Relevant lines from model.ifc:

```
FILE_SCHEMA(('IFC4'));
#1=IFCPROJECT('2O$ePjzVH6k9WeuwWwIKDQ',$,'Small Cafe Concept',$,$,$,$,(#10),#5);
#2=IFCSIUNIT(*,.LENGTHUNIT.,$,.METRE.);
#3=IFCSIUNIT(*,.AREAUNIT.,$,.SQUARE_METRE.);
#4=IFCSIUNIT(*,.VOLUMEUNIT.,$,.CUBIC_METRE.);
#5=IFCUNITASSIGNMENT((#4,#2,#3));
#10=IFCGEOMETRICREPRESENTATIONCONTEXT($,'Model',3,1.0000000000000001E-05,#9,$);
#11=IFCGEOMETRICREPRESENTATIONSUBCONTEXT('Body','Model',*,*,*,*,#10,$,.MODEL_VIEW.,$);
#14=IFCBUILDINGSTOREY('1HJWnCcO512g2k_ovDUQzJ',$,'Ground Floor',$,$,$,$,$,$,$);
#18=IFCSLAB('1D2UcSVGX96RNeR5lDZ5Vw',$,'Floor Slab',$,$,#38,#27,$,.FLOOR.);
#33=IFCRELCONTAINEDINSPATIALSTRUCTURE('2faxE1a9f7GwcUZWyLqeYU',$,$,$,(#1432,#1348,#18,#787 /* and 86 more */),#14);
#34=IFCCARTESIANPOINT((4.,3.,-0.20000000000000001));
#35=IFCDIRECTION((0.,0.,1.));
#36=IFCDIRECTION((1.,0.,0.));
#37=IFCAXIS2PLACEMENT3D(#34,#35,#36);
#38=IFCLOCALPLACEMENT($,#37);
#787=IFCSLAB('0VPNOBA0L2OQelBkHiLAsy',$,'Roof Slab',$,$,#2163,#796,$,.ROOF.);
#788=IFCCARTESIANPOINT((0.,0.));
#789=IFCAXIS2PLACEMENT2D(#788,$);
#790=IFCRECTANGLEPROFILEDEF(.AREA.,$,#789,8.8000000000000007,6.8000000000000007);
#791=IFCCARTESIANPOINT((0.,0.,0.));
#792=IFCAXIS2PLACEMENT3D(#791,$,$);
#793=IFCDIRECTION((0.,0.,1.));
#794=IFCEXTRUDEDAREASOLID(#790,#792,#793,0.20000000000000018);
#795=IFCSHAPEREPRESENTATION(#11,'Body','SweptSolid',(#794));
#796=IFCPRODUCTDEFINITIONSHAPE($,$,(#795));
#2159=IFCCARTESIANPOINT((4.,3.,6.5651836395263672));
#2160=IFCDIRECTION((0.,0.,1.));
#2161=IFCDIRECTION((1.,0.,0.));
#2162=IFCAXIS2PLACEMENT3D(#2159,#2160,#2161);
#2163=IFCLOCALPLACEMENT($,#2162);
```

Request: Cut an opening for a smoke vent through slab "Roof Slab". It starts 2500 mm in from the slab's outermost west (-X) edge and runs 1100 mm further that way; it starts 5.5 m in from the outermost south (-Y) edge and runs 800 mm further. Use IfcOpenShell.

```python
import numpy as np
import ifcopenshell
import ifcopenshell.api.feature
import ifcopenshell.api.geometry
import ifcopenshell.api.root
import ifcopenshell.geom
import ifcopenshell.util.placement
import ifcopenshell.util.representation
import ifcopenshell.util.shape
import ifcopenshell.util.unit

model = ifcopenshell.open("model.ifc")
unit_scale = ifcopenshell.util.unit.calculate_unit_scale(model)
settings = ifcopenshell.geom.settings()


def volume(element):
    """Net volume in cubic metres, openings subtracted."""
    shape = ifcopenshell.geom.create_shape(settings, element)
    return ifcopenshell.util.shape.get_volume(shape.geometry)


slab = model.by_guid("0VPNOBA0L2OQelBkHiLAsy")
before = volume(slab)

# Extent in the slab's own axes, in metres. The edges named are its -X and -Y sides.
slab_shape = ifcopenshell.geom.create_shape(settings, slab)
vertices = ifcopenshell.util.shape.get_vertices(slab_shape.geometry)
x_min, y_min, bottom = vertices.min(axis=0)
top = vertices[:, 2].max()

opening = ifcopenshell.api.root.create_entity(model, ifc_class="IfcOpeningElement", name="Smoke vent opening", predefined_type="OPENING")
context = ifcopenshell.util.representation.get_context(model, "Model", "Body", "MODEL_VIEW")
width, depth = 1.1, 0.8
outline = [(0.0, 0.0), (width, 0.0), (width, depth), (0.0, depth), (0.0, 0.0)]
# Overshoot both faces by 50 mm so the cut is clean.
shape = ifcopenshell.api.geometry.add_slab_representation(
    model, context=context, depth=top - bottom + 0.1, polyline=outline
)
ifcopenshell.api.geometry.assign_representation(model, product=opening, representation=shape)

matrix = ifcopenshell.util.placement.get_local_placement(slab.ObjectPlacement)
matrix[:, 3] = matrix @ np.append(np.array([x_min + 2.5, y_min + 5.5, bottom - 0.05]) / unit_scale, 1.0)
ifcopenshell.api.geometry.edit_object_placement(model, product=opening, matrix=matrix, is_si=False)
ifcopenshell.api.feature.add_feature(model, feature=opening, element=slab)

after = volume(slab)

print(f"slab volume {before:.3f} -> {after:.3f} m3")

model.write("model_edited.ifc")
```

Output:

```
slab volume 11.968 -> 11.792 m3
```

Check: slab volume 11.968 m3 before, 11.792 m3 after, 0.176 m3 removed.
